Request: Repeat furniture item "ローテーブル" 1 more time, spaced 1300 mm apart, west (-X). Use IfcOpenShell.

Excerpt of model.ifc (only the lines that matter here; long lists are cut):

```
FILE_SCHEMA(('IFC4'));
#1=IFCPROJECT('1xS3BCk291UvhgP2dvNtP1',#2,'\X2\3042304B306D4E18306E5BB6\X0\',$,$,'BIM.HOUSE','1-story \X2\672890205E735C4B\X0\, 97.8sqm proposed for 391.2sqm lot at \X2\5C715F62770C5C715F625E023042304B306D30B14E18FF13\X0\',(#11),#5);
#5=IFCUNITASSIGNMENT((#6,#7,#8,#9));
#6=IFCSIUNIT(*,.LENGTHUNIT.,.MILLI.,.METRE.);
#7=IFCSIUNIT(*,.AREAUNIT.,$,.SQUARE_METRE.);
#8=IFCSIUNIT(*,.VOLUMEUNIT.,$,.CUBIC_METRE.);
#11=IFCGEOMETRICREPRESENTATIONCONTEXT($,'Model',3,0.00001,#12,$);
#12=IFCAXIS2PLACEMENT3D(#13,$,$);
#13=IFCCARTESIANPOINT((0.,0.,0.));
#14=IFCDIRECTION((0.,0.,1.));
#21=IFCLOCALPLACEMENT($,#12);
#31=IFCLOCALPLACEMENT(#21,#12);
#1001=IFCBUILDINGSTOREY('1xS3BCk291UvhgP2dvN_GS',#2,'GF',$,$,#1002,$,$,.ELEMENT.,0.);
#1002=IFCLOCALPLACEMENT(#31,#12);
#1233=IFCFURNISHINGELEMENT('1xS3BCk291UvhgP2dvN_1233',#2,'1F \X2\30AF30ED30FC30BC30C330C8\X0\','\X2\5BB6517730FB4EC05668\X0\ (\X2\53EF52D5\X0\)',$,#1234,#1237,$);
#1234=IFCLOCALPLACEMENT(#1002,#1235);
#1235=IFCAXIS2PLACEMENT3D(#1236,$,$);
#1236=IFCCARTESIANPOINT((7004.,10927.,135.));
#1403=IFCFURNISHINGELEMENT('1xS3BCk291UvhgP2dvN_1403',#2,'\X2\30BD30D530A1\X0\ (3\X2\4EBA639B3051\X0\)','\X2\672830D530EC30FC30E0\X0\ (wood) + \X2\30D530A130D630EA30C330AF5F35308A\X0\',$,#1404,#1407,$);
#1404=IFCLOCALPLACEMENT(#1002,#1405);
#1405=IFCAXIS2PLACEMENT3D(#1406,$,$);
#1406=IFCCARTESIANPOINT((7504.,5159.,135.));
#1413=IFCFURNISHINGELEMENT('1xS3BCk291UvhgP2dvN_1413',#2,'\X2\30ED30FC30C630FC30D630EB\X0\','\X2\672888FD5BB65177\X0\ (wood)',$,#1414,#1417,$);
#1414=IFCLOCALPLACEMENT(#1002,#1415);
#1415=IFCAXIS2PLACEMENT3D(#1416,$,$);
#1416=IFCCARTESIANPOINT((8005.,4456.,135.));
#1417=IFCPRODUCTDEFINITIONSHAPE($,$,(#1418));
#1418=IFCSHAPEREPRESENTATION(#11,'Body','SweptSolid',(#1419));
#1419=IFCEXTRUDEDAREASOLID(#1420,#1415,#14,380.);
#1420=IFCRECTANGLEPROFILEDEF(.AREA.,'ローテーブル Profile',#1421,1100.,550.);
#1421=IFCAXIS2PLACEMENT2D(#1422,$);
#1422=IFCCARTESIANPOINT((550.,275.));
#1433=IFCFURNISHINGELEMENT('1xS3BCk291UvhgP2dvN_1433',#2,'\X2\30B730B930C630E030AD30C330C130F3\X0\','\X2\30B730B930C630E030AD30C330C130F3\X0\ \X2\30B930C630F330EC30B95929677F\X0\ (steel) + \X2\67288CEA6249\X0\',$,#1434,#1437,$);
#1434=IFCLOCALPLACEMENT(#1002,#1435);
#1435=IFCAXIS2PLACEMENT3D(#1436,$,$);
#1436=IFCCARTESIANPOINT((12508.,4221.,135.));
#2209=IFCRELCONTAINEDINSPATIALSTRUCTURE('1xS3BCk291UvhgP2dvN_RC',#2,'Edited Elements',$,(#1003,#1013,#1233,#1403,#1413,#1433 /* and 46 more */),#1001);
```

```python
import numpy as np
import ifcopenshell
import ifcopenshell.api.geometry
import ifcopenshell.api.root
import ifcopenshell.util.element
import ifcopenshell.util.placement

model = ifcopenshell.open("model.ifc")


def reuse_history(source, copy):
    """copy_class also copies each property set's owner history, people and application; keep the originals."""
    for rel in copy.IsDefinedBy:
        if rel.is_a("IfcRelDefinesByProperties") and (history := rel.RelatingPropertyDefinition.OwnerHistory):
            rel.RelatingPropertyDefinition.OwnerHistory = source.OwnerHistory
            ifcopenshell.util.element.remove_deep2(model, history)


source = model.by_guid("1xS3BCk291UvhgP2dvN_1413")
base = ifcopenshell.util.placement.get_local_placement(source.ObjectPlacement)
step = np.array([-1.0, 0.0, 0.0]) * 1300.0

for i in range(1, 2):
    copy = ifcopenshell.api.root.copy_class(model, product=source)
    copy.Representation = ifcopenshell.util.element.copy_deep(
        model, source.Representation, exclude=["IfcGeometricRepresentationContext", "IfcRepresentationMap"]
    )
    reuse_history(source, copy)
    matrix = base.copy()
    matrix[:3, 3] += i * step
    print("added at", matrix[:3, 3].round(3) + 0.0)
    ifcopenshell.api.geometry.edit_object_placement(model, product=copy, matrix=matrix, is_si=False)

model.write("model_updated.ifc")
```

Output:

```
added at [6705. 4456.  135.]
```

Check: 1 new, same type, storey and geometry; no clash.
